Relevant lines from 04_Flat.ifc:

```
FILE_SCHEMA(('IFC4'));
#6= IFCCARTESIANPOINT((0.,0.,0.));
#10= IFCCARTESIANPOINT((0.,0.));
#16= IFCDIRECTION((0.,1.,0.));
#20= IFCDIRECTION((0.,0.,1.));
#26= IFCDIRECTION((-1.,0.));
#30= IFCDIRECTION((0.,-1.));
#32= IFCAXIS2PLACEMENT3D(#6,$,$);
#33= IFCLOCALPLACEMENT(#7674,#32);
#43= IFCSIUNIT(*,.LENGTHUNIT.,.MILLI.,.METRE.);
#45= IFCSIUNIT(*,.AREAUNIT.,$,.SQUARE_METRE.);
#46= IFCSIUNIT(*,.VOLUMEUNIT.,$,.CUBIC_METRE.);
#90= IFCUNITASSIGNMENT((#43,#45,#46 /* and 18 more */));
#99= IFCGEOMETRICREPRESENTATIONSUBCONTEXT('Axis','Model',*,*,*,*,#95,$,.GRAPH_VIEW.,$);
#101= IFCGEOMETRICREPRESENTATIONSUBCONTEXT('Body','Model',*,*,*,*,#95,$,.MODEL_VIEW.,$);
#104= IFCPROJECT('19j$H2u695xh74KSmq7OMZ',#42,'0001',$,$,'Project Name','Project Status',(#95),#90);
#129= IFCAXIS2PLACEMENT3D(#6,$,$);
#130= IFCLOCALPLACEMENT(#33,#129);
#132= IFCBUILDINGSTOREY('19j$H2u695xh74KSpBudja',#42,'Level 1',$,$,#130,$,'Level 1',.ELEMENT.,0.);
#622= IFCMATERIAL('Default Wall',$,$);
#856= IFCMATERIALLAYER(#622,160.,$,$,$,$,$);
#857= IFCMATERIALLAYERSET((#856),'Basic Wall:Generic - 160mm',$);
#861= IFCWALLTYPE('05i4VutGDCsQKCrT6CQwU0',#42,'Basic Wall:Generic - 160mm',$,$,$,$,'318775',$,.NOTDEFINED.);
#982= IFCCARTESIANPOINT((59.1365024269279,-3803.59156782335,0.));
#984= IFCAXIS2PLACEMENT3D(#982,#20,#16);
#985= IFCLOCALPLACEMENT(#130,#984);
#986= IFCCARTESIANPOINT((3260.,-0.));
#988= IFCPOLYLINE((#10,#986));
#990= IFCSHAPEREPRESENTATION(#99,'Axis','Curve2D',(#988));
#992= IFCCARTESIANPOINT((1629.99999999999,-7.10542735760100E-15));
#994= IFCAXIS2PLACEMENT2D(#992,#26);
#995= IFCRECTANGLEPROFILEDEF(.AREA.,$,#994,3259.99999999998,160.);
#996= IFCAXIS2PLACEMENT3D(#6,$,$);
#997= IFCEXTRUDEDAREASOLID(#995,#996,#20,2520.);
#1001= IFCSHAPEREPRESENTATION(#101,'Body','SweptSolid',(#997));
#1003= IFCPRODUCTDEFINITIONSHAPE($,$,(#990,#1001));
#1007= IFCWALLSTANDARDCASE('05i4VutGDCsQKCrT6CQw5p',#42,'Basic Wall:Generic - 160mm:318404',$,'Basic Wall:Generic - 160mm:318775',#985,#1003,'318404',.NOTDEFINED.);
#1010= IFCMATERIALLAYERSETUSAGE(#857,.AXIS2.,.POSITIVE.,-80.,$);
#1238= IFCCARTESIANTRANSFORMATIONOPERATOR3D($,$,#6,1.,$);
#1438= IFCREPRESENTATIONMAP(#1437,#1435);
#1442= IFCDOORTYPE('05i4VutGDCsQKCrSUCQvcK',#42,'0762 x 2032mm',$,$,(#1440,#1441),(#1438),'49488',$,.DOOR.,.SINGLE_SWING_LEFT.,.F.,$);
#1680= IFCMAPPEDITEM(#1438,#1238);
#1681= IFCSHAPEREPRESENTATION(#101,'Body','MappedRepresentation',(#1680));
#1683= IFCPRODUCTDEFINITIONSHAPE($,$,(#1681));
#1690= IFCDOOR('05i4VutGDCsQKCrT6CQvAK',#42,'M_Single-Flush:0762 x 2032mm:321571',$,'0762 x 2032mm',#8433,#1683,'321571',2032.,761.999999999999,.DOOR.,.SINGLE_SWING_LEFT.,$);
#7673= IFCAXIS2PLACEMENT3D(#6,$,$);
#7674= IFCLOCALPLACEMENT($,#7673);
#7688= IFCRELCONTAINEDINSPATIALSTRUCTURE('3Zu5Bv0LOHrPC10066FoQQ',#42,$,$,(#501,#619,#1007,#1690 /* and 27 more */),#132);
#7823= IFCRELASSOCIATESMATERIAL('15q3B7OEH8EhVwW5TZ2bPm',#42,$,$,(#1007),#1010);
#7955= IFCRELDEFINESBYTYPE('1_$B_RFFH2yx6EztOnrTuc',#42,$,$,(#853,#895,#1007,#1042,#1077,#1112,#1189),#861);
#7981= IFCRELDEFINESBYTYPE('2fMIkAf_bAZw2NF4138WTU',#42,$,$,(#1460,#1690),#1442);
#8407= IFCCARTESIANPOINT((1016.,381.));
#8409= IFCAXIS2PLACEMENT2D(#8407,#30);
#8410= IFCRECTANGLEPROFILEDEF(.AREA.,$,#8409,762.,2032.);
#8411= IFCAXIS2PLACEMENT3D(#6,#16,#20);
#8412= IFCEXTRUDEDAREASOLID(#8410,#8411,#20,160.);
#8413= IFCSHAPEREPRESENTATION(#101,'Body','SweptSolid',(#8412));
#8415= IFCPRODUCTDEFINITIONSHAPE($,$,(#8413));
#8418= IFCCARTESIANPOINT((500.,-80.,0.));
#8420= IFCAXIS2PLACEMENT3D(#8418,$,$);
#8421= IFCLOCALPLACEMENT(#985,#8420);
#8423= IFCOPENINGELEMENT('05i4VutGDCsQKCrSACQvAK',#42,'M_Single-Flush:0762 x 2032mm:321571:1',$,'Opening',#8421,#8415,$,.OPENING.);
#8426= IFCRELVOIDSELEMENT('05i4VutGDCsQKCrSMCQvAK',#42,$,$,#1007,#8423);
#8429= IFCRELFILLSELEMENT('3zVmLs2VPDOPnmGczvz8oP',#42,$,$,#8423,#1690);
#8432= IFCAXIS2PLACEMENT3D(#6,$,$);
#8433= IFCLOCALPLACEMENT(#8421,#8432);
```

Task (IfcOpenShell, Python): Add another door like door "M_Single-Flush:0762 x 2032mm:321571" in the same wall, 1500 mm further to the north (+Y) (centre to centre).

```python
import ifcopenshell
import ifcopenshell.api.feature
import ifcopenshell.api.geometry
import ifcopenshell.api.root
import ifcopenshell.geom
import ifcopenshell.util.element
import ifcopenshell.util.placement
import ifcopenshell.util.shape

model = ifcopenshell.open("04_Flat.ifc")
settings = ifcopenshell.geom.settings()


def volume(element):
    """Net volume in cubic metres, openings subtracted."""
    shape = ifcopenshell.geom.create_shape(settings, element)
    return ifcopenshell.util.shape.get_volume(shape.geometry)


def reuse_history(source, copy):
    """copy_class also copies each property set's owner history, people and application; keep the originals."""
    for rel in copy.IsDefinedBy:
        if rel.is_a("IfcRelDefinesByProperties") and (history := rel.RelatingPropertyDefinition.OwnerHistory):
            rel.RelatingPropertyDefinition.OwnerHistory = source.OwnerHistory
            ifcopenshell.util.element.remove_deep2(model, history)


door = model.by_guid("05i4VutGDCsQKCrT6CQvAK")
opening = door.FillsVoids[0].RelatingOpeningElement
wall = opening.VoidsElements[0].RelatingBuildingElement
before = volume(wall)
shift = ifcopenshell.util.placement.get_local_placement(wall.ObjectPlacement)[:3, 0] * 1500.0

# copy_class copies the void relationship, type, container and properties, but no geometry.
new_opening = ifcopenshell.api.root.copy_class(model, product=opening)
new_opening.Representation = ifcopenshell.util.element.copy_deep(
    model, opening.Representation, exclude=["IfcGeometricRepresentationContext", "IfcRepresentationMap"]
)
new_opening.Name = "M_Single-Flush:0762 x 2032mm"
new_door = ifcopenshell.api.root.copy_class(model, product=door)
new_door.Representation = ifcopenshell.util.element.copy_deep(
    model, door.Representation, exclude=["IfcGeometricRepresentationContext", "IfcRepresentationMap"]
)
new_door.Name = "M_Single-Flush:0762 x 2032mm"
new_door.Tag = None
reuse_history(door, new_door)
ifcopenshell.api.feature.add_filling(model, opening=new_opening, element=new_door)

for old, new in ((opening, new_opening), (door, new_door)):
    matrix = ifcopenshell.util.placement.get_local_placement(old.ObjectPlacement)
    matrix[:3, 3] += shift
    ifcopenshell.api.geometry.edit_object_placement(model, product=new, matrix=matrix, is_si=False)

after = volume(wall)

print(f"wall volume {before:.3f} -> {after:.3f} m3")

model.write("04_Flat_edited.ifc")
```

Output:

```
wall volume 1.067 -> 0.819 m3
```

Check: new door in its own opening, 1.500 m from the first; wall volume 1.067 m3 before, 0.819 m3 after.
